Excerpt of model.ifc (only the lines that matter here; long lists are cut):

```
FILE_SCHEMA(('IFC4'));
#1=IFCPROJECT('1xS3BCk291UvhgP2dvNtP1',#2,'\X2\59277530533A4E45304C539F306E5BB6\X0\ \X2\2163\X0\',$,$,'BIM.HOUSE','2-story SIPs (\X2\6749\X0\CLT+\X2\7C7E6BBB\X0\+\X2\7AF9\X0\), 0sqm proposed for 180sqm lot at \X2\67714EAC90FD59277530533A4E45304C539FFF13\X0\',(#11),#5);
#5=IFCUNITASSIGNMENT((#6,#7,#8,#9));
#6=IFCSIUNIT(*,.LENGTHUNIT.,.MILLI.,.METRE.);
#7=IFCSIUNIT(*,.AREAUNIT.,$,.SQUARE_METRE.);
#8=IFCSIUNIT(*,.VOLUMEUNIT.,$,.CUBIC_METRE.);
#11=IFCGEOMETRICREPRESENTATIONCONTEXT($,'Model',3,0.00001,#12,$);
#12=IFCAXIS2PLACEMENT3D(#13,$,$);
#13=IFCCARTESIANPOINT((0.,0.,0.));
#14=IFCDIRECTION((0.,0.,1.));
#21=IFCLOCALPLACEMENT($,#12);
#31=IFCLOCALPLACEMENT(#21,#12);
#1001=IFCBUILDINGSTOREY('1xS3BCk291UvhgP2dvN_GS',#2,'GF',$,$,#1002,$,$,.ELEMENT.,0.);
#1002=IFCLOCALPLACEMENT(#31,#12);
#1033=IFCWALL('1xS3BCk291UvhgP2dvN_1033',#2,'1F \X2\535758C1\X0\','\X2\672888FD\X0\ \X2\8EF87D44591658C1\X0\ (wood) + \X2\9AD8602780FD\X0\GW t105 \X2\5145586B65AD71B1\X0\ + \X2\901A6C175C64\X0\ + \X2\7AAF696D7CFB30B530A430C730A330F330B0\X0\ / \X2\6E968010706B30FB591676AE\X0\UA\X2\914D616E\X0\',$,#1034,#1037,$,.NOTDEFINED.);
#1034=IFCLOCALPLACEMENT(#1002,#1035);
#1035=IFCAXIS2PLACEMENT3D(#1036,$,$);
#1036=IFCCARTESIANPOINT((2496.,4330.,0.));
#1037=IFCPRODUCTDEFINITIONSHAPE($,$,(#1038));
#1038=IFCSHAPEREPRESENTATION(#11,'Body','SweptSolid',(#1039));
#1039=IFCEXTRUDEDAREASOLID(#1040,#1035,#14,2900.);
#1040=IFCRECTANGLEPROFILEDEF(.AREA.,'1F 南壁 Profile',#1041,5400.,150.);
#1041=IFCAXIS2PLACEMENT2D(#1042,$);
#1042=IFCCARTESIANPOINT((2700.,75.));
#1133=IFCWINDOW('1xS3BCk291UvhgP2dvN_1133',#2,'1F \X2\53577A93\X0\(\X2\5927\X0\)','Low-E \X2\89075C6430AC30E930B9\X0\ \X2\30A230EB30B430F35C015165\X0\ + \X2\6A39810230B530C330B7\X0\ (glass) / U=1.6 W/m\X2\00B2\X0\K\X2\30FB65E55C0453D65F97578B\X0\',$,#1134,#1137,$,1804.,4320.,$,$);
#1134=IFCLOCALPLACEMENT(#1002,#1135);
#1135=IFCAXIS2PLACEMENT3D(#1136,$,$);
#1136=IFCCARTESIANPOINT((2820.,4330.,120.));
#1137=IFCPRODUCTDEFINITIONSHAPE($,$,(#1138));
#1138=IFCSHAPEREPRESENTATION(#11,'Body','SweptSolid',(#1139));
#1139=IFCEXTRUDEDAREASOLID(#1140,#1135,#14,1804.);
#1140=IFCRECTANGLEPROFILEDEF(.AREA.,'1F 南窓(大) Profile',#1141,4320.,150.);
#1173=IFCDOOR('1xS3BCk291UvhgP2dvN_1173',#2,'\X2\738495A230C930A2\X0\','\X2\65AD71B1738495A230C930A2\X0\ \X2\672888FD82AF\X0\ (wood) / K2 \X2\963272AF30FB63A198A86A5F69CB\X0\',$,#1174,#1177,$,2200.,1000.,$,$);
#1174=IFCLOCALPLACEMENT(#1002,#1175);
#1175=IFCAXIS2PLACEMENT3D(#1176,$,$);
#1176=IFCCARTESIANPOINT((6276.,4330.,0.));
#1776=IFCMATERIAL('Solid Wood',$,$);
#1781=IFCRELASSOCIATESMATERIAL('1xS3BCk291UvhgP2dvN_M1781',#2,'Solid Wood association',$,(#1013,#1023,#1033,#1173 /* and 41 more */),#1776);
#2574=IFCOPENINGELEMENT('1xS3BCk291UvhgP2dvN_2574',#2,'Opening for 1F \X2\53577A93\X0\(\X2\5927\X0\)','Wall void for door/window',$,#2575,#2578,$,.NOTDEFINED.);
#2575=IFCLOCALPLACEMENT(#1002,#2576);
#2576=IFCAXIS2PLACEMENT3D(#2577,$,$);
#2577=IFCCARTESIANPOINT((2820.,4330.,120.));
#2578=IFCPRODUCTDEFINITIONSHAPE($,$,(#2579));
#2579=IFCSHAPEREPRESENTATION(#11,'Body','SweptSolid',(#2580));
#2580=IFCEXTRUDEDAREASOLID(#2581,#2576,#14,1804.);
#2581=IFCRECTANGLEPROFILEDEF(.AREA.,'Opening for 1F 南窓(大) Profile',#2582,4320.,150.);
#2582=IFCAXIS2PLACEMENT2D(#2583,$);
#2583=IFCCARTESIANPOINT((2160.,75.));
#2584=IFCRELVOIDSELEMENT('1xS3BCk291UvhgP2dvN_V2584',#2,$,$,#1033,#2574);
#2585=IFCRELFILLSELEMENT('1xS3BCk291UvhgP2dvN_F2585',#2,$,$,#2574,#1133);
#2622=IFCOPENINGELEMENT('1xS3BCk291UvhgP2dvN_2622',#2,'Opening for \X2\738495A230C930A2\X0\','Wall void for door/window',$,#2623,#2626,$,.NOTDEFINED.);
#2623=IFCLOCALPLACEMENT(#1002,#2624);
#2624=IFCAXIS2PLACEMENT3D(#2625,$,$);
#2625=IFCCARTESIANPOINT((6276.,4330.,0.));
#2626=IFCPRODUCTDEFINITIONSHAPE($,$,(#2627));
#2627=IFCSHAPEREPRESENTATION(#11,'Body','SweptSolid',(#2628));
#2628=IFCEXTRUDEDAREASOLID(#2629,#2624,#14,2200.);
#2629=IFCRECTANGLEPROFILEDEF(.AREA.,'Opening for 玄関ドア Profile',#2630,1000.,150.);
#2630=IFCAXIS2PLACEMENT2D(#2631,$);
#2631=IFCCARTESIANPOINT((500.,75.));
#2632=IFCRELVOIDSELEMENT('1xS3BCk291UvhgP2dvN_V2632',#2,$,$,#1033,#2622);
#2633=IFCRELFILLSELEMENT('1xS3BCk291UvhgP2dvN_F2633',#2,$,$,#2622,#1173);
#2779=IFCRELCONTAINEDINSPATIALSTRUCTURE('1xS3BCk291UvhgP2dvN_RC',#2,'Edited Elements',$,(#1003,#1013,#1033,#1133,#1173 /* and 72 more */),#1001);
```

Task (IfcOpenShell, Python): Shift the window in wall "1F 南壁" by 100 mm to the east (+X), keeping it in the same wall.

```python
import ifcopenshell
import ifcopenshell.api.geometry
import ifcopenshell.util.placement

model = ifcopenshell.open("model.ifc")

window = model.by_guid("1xS3BCk291UvhgP2dvN_1133")
opening = window.FillsVoids[0].RelatingOpeningElement
wall = opening.VoidsElements[0].RelatingBuildingElement

wall_matrix = ifcopenshell.util.placement.get_local_placement(wall.ObjectPlacement)
shift = wall_matrix[:3, 0] * 100.0
before = ifcopenshell.util.placement.get_local_placement(window.ObjectPlacement)[:3, 3].copy()

# The window is not placed relative to its opening, so move both.
for product in (opening, window):
    matrix = ifcopenshell.util.placement.get_local_placement(product.ObjectPlacement)
    matrix[:3, 3] += shift
    ifcopenshell.api.geometry.edit_object_placement(model, product=product, matrix=matrix, is_si=False)

after = ifcopenshell.util.placement.get_local_placement(window.ObjectPlacement)[:3, 3]
print("window moved by", (after - before).round(3) + 0.0)

model.write("model-out.ifc")
```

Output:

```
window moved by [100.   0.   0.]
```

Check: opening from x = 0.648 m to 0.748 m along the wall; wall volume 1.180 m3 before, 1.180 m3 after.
